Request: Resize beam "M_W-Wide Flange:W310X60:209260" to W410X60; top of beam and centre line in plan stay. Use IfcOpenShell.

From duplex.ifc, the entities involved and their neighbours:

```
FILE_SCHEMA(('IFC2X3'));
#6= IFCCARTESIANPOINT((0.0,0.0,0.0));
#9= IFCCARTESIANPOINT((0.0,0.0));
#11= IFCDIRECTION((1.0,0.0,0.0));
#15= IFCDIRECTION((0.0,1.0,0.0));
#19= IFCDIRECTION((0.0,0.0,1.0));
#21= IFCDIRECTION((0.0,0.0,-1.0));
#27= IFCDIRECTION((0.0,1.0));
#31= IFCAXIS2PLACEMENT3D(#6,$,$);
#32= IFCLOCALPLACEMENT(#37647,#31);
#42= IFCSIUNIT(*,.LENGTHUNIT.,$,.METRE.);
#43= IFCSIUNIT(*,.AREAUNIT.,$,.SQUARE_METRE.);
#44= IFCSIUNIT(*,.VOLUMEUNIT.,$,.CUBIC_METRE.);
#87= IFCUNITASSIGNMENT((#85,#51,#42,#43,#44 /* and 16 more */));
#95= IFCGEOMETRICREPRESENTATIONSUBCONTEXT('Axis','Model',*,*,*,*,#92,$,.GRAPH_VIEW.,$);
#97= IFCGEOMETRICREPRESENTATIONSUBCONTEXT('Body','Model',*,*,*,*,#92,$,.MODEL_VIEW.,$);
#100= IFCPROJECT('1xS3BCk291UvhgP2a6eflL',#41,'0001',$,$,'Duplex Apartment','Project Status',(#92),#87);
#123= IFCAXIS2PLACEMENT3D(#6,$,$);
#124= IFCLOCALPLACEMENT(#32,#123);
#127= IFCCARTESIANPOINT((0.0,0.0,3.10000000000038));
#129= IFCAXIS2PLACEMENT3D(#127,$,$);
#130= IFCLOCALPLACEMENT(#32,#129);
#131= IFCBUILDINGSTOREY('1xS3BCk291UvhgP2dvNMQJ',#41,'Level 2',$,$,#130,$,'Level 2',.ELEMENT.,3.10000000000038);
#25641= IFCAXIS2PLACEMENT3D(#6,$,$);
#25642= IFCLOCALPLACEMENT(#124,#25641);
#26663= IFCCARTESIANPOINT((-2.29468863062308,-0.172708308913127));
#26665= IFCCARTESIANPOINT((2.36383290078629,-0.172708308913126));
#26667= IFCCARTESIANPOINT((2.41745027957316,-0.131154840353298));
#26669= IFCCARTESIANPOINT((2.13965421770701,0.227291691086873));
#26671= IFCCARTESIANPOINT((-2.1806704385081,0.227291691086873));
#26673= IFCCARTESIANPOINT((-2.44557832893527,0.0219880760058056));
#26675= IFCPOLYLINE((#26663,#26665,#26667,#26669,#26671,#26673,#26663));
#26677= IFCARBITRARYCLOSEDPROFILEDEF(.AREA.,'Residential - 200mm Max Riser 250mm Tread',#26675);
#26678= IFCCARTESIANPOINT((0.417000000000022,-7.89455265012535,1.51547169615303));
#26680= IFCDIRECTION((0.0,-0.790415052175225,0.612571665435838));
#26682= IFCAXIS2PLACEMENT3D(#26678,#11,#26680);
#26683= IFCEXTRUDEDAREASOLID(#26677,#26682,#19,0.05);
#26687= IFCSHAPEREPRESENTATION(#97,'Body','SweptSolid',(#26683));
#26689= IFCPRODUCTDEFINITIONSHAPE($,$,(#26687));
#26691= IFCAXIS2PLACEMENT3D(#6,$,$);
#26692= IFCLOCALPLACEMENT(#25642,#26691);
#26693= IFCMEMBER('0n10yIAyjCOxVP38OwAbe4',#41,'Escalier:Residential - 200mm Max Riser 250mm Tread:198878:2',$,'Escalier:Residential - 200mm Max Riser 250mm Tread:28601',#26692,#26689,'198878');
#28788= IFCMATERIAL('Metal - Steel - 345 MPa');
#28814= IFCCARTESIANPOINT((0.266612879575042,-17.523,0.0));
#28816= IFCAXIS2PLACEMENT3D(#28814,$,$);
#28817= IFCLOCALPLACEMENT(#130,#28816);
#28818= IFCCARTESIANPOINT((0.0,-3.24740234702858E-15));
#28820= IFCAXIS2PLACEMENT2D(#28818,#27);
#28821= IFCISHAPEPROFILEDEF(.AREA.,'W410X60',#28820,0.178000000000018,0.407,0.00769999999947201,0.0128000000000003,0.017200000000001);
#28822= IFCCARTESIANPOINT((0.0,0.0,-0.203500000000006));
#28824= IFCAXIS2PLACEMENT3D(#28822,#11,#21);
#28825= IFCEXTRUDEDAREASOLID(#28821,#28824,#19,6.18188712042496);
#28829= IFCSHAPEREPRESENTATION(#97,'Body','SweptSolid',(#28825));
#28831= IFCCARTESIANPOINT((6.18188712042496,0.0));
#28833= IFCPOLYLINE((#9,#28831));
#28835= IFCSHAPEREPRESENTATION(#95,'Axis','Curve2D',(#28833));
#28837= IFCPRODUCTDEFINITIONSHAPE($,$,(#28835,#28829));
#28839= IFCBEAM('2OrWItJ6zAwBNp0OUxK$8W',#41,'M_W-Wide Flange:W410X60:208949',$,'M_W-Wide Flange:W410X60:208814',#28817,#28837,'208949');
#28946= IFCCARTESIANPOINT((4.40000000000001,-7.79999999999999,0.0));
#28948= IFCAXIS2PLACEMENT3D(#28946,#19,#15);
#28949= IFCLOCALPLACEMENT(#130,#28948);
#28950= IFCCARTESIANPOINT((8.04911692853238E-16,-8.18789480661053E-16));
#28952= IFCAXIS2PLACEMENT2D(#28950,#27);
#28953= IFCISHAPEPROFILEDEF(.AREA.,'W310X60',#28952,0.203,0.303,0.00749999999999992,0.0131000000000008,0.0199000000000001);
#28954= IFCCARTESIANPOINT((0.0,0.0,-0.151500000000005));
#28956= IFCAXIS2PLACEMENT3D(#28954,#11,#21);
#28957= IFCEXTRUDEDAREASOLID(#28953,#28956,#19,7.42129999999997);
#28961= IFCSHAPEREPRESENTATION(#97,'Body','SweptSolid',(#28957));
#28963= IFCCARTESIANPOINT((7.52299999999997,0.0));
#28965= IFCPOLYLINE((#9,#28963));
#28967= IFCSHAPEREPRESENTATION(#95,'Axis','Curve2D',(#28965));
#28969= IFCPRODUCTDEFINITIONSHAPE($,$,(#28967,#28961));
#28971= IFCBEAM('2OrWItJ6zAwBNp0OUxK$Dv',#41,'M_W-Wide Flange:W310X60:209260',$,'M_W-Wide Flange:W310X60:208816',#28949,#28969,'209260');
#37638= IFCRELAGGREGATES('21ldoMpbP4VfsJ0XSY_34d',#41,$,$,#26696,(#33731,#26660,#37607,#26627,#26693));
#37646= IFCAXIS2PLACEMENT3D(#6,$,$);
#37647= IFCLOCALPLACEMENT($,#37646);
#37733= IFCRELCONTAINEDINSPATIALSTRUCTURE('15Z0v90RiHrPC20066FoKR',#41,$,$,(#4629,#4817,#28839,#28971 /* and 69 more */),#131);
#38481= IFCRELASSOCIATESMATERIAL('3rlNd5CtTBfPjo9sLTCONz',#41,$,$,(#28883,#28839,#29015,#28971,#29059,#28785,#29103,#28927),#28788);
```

```python
import ifcopenshell
import ifcopenshell.util.element
import ifcopenshell.util.representation

model = ifcopenshell.open("duplex.ifc")

member = model.by_id(28971)
source = next(p for p in model.by_type("IfcIShapeProfileDef") if p.ProfileName == "W410X60")

body = ifcopenshell.util.representation.get_representation(member, "Model", "Body")
solid = body.Items[0]
old_profile = solid.SweptArea

# Copy the section's sizes but keep this member's own profile position.
profile = ifcopenshell.util.element.copy(model, source)
# Profiles are centred, so shift by half the change in depth to hold the top.
shift = (old_profile.OverallDepth - profile.OverallDepth) / 2
x, y = old_profile.Position.Location.Coordinates
up = (-1.0, 0.0)  # upwards, in the solid's own plane
location = model.createIfcCartesianPoint((x + up[0] * shift, y + up[1] * shift))
profile.Position = model.createIfcAxis2Placement2D(location, old_profile.Position.RefDirection)
solid.SweptArea = profile
if not model.get_total_inverses(old_profile):
    ifcopenshell.util.element.remove_deep2(model, old_profile)
member.Name = member.Name.replace("W310X60", "W410X60")
member.ObjectType = member.ObjectType.replace("W310X60", "W410X60")

print(solid.SweptArea)

model.write("duplex_v2.ifc")
```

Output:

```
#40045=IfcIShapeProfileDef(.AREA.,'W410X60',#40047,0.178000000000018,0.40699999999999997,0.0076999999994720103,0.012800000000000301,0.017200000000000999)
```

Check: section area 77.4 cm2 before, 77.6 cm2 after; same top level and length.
